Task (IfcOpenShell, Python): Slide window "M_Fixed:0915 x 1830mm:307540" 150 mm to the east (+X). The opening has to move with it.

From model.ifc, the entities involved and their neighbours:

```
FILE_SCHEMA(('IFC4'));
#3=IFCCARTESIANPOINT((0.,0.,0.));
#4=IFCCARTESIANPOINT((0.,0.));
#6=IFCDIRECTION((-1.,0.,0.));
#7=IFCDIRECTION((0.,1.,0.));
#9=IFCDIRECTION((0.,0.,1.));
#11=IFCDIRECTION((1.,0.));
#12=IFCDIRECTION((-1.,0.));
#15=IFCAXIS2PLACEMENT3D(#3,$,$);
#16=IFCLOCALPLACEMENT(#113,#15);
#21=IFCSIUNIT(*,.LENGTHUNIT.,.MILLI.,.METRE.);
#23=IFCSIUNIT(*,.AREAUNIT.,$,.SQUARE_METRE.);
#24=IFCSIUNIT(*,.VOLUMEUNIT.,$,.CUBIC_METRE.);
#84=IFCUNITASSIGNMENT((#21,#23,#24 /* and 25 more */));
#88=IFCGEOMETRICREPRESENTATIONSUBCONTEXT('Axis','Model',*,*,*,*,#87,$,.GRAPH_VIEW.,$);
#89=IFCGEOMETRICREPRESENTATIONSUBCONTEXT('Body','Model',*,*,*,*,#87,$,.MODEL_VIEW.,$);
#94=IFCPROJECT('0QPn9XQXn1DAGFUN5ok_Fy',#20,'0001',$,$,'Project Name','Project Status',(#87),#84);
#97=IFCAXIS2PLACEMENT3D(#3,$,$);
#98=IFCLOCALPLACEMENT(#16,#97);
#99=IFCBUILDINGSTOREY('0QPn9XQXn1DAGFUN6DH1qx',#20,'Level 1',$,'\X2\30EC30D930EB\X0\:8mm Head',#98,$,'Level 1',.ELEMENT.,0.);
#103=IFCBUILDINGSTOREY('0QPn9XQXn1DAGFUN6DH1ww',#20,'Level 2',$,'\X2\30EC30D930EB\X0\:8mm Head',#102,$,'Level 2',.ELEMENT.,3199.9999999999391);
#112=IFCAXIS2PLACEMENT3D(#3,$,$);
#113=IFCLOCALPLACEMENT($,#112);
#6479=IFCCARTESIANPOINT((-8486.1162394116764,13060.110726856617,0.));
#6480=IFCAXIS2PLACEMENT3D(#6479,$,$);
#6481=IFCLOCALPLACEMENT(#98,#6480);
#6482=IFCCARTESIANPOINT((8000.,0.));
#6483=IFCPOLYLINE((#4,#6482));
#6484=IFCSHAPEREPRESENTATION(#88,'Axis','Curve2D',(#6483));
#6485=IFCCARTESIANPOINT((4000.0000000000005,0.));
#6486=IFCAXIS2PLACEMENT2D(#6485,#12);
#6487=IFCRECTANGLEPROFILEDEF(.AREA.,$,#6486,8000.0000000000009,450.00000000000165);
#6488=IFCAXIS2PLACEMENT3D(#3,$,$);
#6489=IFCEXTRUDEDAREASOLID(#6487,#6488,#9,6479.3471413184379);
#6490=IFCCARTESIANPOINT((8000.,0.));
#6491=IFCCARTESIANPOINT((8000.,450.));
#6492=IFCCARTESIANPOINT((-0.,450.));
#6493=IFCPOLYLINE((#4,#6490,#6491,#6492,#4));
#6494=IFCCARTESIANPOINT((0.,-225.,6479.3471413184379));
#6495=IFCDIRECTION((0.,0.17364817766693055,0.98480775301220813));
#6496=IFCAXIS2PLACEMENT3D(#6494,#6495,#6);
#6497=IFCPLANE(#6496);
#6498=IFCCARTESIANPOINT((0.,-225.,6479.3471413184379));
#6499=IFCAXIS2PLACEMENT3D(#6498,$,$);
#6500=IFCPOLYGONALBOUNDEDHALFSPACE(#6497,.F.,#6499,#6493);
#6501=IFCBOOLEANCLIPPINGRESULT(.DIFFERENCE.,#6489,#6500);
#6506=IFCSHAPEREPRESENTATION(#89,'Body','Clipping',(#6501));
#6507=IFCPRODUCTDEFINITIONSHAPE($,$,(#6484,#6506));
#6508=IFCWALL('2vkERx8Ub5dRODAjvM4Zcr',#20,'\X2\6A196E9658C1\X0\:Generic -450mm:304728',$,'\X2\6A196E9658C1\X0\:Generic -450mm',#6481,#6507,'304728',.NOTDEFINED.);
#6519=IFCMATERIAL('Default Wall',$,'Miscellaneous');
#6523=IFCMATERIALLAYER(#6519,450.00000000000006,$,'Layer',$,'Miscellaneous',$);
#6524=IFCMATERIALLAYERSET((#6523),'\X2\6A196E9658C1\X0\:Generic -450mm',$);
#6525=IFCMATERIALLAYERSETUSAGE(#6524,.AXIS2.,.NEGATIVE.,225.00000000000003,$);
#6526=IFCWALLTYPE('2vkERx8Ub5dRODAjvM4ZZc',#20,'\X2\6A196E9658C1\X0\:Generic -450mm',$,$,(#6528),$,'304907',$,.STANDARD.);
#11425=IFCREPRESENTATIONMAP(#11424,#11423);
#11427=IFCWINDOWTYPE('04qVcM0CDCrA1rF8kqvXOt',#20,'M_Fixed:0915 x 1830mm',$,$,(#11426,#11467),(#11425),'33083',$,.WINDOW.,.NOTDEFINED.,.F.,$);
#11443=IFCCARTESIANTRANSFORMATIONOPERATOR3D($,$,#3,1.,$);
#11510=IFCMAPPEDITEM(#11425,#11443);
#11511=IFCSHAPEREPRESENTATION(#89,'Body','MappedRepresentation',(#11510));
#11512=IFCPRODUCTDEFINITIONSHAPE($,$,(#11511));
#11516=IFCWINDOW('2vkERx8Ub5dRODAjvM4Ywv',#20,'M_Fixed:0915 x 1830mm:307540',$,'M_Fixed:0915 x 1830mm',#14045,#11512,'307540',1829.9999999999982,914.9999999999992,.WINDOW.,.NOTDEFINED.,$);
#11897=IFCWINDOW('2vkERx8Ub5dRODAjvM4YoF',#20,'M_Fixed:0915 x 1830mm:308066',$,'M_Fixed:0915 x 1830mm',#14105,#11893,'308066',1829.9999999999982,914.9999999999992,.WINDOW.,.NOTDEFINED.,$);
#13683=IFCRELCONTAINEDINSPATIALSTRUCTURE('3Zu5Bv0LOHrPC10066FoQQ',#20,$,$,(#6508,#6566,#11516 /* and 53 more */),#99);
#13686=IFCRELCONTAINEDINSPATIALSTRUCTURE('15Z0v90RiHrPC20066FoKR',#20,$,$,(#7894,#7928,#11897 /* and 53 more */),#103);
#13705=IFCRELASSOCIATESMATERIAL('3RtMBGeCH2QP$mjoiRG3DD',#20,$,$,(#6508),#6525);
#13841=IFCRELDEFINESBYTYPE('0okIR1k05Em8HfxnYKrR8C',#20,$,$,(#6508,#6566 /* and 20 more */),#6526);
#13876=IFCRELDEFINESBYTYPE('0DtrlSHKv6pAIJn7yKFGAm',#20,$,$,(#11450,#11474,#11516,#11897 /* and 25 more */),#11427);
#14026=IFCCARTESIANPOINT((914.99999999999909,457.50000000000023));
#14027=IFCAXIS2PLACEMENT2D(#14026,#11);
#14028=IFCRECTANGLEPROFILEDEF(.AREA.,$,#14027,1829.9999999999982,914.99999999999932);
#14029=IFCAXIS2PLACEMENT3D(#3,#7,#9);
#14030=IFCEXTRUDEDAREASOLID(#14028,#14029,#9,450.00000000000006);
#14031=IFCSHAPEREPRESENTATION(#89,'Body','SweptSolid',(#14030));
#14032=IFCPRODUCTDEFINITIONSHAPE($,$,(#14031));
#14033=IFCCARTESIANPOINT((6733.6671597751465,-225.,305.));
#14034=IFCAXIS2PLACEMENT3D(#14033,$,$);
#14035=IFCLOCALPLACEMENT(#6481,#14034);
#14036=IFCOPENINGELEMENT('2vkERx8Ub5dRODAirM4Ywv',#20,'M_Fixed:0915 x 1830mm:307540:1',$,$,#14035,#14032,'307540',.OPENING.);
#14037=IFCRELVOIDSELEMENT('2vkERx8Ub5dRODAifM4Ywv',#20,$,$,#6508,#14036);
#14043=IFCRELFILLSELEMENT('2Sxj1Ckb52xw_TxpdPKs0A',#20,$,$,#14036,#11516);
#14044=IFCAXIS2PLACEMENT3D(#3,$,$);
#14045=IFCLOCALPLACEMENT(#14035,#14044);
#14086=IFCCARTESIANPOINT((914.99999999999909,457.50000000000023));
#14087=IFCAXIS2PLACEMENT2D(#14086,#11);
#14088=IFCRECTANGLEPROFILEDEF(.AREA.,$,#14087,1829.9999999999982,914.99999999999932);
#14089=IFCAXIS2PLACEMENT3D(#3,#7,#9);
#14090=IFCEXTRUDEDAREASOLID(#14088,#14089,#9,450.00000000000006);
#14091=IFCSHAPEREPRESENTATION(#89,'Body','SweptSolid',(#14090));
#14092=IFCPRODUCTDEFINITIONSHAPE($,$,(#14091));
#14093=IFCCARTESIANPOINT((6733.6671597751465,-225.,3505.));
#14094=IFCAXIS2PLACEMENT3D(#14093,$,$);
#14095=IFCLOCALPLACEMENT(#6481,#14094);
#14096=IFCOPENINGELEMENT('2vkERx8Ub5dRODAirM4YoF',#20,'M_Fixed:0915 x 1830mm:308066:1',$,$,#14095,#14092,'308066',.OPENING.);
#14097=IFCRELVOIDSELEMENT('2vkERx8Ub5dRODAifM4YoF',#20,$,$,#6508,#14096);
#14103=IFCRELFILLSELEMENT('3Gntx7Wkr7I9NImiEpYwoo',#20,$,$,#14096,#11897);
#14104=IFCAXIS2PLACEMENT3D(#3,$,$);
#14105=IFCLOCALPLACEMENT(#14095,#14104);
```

```python
import ifcopenshell
import ifcopenshell.api.geometry
import ifcopenshell.util.placement
import ifcopenshell.util.unit

model = ifcopenshell.open("model.ifc")
unit_scale = ifcopenshell.util.unit.calculate_unit_scale(model)

window = model.by_guid("2vkERx8Ub5dRODAjvM4Ywv")
opening = window.FillsVoids[0].RelatingOpeningElement
wall = opening.VoidsElements[0].RelatingBuildingElement

wall_matrix = ifcopenshell.util.placement.get_local_placement(wall.ObjectPlacement)
shift = wall_matrix[:3, 0] * 0.15 / unit_scale
before = ifcopenshell.util.placement.get_local_placement(window.ObjectPlacement)[:3, 3].copy()

# The window is placed relative to its opening, so it follows when the opening moves.
matrix = ifcopenshell.util.placement.get_local_placement(opening.ObjectPlacement)
matrix[:3, 3] += shift
ifcopenshell.api.geometry.edit_object_placement(
    model, product=opening, matrix=matrix, is_si=False, should_transform_children=True
)

after = ifcopenshell.util.placement.get_local_placement(window.ObjectPlacement)[:3, 3]
print("window moved by", (after - before).round(3) + 0.0)

model.write("model-out.ifc")
```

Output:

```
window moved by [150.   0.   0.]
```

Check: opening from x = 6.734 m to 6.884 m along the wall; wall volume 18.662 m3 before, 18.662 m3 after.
